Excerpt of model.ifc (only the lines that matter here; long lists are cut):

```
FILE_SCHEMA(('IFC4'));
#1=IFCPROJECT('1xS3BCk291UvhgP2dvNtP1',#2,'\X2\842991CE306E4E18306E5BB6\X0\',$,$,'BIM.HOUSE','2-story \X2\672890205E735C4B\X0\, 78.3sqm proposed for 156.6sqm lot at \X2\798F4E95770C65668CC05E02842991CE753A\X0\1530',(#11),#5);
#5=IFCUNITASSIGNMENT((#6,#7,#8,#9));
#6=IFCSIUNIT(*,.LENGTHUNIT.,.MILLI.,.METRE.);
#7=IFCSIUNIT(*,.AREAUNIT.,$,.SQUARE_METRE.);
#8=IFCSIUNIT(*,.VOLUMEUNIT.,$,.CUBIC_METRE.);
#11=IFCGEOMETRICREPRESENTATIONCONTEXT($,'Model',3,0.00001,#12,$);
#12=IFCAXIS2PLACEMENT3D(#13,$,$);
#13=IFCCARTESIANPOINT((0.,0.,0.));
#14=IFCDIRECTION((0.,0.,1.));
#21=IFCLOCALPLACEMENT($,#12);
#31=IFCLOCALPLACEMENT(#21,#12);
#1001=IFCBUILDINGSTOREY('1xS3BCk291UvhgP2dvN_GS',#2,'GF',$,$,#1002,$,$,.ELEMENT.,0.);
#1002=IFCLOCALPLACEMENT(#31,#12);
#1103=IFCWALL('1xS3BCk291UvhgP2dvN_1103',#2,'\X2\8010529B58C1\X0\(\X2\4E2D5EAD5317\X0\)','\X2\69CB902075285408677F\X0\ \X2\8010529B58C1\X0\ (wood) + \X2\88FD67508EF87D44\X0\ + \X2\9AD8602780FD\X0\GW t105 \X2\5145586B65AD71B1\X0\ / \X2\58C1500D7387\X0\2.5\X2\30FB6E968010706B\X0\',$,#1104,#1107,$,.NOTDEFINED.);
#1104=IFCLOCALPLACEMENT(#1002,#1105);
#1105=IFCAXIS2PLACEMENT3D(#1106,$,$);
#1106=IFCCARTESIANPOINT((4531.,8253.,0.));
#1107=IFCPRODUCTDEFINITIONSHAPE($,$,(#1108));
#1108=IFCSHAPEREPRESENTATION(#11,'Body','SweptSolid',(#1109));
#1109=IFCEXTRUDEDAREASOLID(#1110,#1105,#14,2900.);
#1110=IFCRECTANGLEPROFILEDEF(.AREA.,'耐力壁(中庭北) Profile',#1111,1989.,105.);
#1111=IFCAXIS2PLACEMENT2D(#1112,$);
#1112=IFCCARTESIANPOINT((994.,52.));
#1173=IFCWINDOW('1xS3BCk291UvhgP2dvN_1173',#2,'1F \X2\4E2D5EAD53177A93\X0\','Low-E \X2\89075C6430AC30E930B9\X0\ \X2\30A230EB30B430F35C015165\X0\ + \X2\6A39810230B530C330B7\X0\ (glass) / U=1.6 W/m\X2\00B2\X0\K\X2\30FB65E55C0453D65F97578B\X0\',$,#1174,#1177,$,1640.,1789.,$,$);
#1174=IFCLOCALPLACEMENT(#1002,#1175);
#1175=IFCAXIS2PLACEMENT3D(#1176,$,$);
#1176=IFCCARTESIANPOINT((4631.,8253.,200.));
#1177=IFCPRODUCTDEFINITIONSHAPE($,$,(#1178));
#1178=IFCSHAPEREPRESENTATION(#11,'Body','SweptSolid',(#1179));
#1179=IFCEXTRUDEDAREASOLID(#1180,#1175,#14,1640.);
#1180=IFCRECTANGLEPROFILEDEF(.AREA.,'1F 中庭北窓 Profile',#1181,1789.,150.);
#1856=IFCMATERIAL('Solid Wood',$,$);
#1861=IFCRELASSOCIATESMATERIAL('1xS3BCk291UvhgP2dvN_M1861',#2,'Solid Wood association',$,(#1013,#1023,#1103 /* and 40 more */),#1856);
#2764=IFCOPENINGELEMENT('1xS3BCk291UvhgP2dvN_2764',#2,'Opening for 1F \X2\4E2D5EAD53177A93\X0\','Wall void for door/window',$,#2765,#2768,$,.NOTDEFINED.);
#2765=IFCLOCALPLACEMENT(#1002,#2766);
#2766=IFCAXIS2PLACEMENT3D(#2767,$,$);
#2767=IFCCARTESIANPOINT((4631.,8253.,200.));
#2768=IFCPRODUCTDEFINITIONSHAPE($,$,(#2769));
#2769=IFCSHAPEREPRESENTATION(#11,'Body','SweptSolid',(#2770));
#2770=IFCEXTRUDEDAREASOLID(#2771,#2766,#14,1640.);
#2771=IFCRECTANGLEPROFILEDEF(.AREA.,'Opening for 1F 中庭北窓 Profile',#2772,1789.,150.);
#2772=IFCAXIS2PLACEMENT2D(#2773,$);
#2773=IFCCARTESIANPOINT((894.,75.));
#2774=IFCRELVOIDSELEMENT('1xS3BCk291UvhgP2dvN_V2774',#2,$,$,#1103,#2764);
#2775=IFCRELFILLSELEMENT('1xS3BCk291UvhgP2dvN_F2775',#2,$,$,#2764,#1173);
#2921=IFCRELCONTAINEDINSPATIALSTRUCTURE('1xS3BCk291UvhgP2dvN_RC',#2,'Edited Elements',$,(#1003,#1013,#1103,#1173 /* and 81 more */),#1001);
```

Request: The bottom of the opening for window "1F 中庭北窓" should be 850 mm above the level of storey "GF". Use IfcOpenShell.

```python
import numpy as np
import ifcopenshell
import ifcopenshell.api.geometry
import ifcopenshell.geom
import ifcopenshell.util.element
import ifcopenshell.util.placement
import ifcopenshell.util.shape
import ifcopenshell.util.unit

model = ifcopenshell.open("model.ifc")
unit_scale = ifcopenshell.util.unit.calculate_unit_scale(model)

window = model.by_guid("1xS3BCk291UvhgP2dvN_1173")
opening = window.FillsVoids[0].RelatingOpeningElement
storey = ifcopenshell.util.element.get_container(window, ifc_class="IfcBuildingStorey")
level = ifcopenshell.util.placement.get_local_placement(storey.ObjectPlacement)[2, 3]

# The opening's origin need not be at the sill, so measure its lowest point.
shape = ifcopenshell.geom.create_shape(ifcopenshell.geom.settings(), opening)
bottom = ifcopenshell.util.shape.get_shape_bottom_elevation(shape, shape.geometry) / unit_scale
dz = level + 850.0 - bottom

shift = np.array([0.0, 0.0, dz])
# The window is not placed relative to its opening, so move both.
for product in (opening, window):
    matrix = ifcopenshell.util.placement.get_local_placement(product.ObjectPlacement)
    matrix[:3, 3] += shift
    ifcopenshell.api.geometry.edit_object_placement(model, product=product, matrix=matrix, is_si=False)

print(f"moved by {dz * unit_scale:+.3f} m")

model.write("model_edited.ifc")
```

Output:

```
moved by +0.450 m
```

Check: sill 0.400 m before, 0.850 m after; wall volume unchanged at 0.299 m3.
